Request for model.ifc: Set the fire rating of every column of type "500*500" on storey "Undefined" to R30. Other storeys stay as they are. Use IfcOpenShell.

First a look at what the model holds.

```python
import ifcopenshell
import ifcopenshell.util.element

model = ifcopenshell.open("model.ifc")
print(model.schema)
storey = next(s for s in model.by_type("IfcBuildingStorey") if s.Name == "Undefined")
columns = [e for e in ifcopenshell.util.element.get_decomposition(storey) if e.is_a("IfcColumn")]
seen = {}
for e in columns:
    element_type = ifcopenshell.util.element.get_type(e)
    key = (element_type.Name if element_type != e and element_type else None, ifcopenshell.util.element.get_pset(e, "Pset_ColumnCommon", "FireRating"))
    seen[key] = seen.get(key, 0) + 1
for (name, value), count in sorted(seen.items(), key=str):
    print(count, "x", name, "|", value)
```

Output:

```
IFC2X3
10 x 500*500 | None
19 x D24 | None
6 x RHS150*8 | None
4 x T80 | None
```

```python
import ifcopenshell
import ifcopenshell.api.pset
import ifcopenshell.util.element

model = ifcopenshell.open("model.ifc")

storey = next(s for s in model.by_type("IfcBuildingStorey") if s.Name == "Undefined")
columns = [e for e in ifcopenshell.util.element.get_decomposition(storey) if e.is_a("IfcColumn")]

count = 0
for e in columns:
    element_type = ifcopenshell.util.element.get_type(e)
    if element_type in (None, e) or element_type.Name != "500*500":
        continue
    # add_pset returns the element's existing set when there is one.
    pset = ifcopenshell.api.pset.add_pset(model, product=e, name="Pset_ColumnCommon")
    ifcopenshell.api.pset.edit_pset(model, pset=pset, properties={"FireRating": "R30"})
    count += 1

print(count, "columns updated")

model.write("model_rev.ifc")
```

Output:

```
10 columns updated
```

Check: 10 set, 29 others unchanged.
